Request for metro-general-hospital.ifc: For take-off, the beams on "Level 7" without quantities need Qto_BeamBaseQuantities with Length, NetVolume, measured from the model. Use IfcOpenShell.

First a look at what the model holds.

```python
import ifcopenshell
import ifcopenshell.util.element
import ifcopenshell.util.unit

model = ifcopenshell.open("metro-general-hospital.ifc")
print(model.schema)
for unit_type in ("LENGTHUNIT", "AREAUNIT", "VOLUMEUNIT"):
    print(unit_type, ifcopenshell.util.unit.calculate_unit_scale(model, unit_type))
storey = next(s for s in model.by_type("IfcBuildingStorey") if s.Name == "Level 7")
beams = [e for e in ifcopenshell.util.element.get_decomposition(storey) if e.is_a("IfcBeam")]
for e in sorted(beams, key=lambda e: e.id()):
    print(e.id(), e.is_a(), e.Name, list(ifcopenshell.util.element.get_psets(e, qtos_only=True)), sep=" | ")
```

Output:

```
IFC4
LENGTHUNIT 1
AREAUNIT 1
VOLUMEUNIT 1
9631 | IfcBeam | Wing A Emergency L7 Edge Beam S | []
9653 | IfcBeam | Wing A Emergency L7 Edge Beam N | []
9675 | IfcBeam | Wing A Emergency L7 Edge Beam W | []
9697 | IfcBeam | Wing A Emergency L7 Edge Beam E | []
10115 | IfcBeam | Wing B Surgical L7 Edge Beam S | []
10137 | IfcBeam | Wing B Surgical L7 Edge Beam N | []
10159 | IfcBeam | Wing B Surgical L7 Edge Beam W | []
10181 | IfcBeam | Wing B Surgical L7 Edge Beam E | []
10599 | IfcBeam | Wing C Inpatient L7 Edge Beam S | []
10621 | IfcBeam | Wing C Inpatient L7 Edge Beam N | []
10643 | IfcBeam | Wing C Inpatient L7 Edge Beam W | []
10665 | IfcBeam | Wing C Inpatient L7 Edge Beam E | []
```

```python
import ifcopenshell
import ifcopenshell.api.pset
import ifcopenshell.geom
import ifcopenshell.util.element
import ifcopenshell.util.shape
import ifcopenshell.util.unit

model = ifcopenshell.open("metro-general-hospital.ifc")
unit_scale = ifcopenshell.util.unit.calculate_unit_scale(model)
volume_scale = ifcopenshell.util.unit.calculate_unit_scale(model, "VOLUMEUNIT")
settings = ifcopenshell.geom.settings()

storey = next(s for s in model.by_type("IfcBuildingStorey") if s.Name == "Level 7")
beams = [e for e in ifcopenshell.util.element.get_decomposition(storey) if e.is_a("IfcBeam")]

for e in sorted(beams, key=lambda e: e.id()):
    if ifcopenshell.util.element.get_psets(e, qtos_only=True, should_inherit=False):
        continue
    # Geometry comes back in metres, in the element's own axes.
    shape = ifcopenshell.geom.create_shape(settings, e)
    values = {
        "Length": ifcopenshell.util.shape.get_max_xyz(shape.geometry) / unit_scale,
        "NetVolume": ifcopenshell.util.shape.get_volume(shape.geometry) / volume_scale,
    }
    qto = ifcopenshell.api.pset.add_qto(model, product=e, name="Qto_BeamBaseQuantities")
    ifcopenshell.api.pset.edit_qto(model, qto=qto, properties=values)
    print(e.id(), {k: round(v, 3) for k, v in values.items()})

model.write("metro-general-hospital-out.ifc")
```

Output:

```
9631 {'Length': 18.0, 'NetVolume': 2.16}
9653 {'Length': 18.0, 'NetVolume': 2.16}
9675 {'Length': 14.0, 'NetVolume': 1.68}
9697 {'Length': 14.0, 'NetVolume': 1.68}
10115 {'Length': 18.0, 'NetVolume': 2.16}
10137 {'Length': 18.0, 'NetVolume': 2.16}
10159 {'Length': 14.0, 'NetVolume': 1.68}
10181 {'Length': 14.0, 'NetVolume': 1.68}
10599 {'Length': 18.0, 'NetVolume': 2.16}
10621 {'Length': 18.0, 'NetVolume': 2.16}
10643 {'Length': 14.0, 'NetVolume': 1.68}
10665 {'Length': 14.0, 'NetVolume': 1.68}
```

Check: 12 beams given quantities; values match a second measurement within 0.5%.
